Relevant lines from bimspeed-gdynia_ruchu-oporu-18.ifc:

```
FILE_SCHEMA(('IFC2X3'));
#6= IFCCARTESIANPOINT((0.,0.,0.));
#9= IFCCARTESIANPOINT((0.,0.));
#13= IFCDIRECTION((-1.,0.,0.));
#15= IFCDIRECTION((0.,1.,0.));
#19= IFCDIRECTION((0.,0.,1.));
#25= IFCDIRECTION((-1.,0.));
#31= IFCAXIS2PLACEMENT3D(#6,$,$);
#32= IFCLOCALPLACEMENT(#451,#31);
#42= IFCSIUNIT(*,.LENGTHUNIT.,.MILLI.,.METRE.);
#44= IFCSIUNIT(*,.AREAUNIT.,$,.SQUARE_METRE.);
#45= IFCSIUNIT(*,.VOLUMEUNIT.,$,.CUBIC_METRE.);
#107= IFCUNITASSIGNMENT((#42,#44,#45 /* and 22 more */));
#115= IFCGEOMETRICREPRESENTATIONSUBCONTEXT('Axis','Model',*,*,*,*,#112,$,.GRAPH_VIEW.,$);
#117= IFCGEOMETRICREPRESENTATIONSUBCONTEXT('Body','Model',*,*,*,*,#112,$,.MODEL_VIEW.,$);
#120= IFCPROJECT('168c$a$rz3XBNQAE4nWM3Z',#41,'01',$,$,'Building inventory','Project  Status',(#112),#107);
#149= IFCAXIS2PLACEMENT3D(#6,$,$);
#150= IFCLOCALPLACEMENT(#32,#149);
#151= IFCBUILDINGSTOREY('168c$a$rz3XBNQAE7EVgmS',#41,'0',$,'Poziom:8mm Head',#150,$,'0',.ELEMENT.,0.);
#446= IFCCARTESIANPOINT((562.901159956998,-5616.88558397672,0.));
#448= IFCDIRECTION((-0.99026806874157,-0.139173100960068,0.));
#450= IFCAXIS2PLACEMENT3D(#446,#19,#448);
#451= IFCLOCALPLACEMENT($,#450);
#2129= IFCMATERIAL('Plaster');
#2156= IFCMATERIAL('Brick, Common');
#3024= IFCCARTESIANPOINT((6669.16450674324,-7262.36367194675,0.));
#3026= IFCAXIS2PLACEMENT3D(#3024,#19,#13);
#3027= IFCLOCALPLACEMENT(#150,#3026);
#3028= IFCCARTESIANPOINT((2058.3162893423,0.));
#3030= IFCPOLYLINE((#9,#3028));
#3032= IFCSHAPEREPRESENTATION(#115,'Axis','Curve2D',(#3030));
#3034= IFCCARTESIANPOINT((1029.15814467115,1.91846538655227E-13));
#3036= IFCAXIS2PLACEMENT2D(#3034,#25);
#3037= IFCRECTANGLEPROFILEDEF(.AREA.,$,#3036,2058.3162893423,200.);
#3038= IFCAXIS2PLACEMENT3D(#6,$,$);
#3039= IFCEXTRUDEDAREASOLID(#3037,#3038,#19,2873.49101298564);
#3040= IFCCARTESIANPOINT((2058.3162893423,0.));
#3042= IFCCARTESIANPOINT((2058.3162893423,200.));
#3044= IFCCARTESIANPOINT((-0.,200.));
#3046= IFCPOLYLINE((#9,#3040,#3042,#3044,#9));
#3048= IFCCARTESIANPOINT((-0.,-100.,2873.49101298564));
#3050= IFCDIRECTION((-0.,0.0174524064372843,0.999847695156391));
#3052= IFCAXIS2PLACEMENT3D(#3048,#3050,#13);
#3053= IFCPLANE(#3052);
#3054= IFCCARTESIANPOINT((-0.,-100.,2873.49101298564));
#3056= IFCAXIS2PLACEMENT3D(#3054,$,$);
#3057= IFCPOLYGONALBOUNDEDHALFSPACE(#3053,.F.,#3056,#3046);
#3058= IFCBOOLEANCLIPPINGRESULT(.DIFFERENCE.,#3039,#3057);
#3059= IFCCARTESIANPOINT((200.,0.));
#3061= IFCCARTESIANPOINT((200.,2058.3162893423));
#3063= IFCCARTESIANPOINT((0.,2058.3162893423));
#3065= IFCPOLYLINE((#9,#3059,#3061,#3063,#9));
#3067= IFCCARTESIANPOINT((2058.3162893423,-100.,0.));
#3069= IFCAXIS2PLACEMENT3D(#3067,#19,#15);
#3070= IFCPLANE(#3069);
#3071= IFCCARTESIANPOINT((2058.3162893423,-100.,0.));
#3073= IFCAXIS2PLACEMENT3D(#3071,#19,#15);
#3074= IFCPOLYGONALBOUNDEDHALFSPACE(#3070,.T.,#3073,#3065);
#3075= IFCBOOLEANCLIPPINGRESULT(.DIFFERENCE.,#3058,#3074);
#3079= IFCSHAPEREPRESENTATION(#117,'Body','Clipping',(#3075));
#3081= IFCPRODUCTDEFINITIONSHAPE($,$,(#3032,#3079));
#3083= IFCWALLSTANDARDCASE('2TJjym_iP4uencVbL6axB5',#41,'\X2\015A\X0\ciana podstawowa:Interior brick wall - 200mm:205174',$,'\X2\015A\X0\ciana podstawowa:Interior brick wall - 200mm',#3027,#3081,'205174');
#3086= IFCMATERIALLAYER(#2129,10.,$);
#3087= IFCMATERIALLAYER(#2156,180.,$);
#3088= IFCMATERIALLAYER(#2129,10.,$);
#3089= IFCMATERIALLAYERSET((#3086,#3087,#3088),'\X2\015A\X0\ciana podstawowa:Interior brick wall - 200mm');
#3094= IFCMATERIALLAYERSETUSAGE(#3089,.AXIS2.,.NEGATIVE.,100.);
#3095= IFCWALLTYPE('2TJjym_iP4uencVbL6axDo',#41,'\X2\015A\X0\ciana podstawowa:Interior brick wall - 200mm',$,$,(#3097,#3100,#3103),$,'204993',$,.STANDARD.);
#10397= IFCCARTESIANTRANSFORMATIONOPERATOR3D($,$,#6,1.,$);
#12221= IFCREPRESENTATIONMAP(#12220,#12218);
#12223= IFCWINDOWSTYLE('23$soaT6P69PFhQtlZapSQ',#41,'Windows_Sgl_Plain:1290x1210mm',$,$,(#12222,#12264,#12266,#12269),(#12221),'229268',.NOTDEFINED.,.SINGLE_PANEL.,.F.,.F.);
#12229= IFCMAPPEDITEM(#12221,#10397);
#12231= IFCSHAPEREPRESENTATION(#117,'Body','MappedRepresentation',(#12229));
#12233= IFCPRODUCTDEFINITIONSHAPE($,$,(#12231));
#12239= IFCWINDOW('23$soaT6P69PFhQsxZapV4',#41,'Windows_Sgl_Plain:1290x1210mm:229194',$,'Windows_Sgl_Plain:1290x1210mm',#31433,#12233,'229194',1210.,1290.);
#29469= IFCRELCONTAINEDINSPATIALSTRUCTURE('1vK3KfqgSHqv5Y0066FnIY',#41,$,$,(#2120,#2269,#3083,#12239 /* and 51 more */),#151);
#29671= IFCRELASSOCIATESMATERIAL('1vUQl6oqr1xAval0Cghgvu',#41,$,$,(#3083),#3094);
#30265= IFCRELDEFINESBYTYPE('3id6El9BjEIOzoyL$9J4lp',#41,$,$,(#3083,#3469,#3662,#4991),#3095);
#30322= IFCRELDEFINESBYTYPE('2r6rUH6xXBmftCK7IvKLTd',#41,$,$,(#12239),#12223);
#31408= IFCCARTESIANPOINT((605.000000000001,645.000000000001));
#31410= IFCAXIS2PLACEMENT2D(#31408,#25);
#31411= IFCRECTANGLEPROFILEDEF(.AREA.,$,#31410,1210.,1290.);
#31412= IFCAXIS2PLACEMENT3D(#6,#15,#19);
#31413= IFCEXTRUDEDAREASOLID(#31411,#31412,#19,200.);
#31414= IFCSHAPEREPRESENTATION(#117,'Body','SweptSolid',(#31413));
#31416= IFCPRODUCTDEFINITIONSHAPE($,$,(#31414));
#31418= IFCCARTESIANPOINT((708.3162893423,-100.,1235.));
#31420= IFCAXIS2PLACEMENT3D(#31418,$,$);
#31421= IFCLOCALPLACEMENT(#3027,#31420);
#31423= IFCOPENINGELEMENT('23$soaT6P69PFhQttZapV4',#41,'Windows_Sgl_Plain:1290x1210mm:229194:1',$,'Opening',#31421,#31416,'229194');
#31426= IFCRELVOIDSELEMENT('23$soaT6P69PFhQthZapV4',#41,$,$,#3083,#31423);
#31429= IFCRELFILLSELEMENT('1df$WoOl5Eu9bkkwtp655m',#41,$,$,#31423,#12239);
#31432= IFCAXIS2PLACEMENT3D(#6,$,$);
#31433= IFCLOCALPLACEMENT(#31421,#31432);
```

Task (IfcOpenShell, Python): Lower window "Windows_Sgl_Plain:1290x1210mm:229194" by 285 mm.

```python
import numpy as np
import ifcopenshell
import ifcopenshell.api.geometry
import ifcopenshell.util.placement
import ifcopenshell.util.unit

model = ifcopenshell.open("bimspeed-gdynia_ruchu-oporu-18.ifc")
unit_scale = ifcopenshell.util.unit.calculate_unit_scale(model)

window = model.by_guid("23$soaT6P69PFhQsxZapV4")
opening = window.FillsVoids[0].RelatingOpeningElement
dz = -285.0

shift = np.array([0.0, 0.0, dz])
# The window is placed relative to its opening, so it follows when the opening moves.
matrix = ifcopenshell.util.placement.get_local_placement(opening.ObjectPlacement)
matrix[:3, 3] += shift
ifcopenshell.api.geometry.edit_object_placement(
    model, product=opening, matrix=matrix, is_si=False, should_transform_children=True
)

print(f"moved by {dz * unit_scale:+.3f} m")

model.write("bimspeed-gdynia_ruchu-oporu-18_v2.ifc")
```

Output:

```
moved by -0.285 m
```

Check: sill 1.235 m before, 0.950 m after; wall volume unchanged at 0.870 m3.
